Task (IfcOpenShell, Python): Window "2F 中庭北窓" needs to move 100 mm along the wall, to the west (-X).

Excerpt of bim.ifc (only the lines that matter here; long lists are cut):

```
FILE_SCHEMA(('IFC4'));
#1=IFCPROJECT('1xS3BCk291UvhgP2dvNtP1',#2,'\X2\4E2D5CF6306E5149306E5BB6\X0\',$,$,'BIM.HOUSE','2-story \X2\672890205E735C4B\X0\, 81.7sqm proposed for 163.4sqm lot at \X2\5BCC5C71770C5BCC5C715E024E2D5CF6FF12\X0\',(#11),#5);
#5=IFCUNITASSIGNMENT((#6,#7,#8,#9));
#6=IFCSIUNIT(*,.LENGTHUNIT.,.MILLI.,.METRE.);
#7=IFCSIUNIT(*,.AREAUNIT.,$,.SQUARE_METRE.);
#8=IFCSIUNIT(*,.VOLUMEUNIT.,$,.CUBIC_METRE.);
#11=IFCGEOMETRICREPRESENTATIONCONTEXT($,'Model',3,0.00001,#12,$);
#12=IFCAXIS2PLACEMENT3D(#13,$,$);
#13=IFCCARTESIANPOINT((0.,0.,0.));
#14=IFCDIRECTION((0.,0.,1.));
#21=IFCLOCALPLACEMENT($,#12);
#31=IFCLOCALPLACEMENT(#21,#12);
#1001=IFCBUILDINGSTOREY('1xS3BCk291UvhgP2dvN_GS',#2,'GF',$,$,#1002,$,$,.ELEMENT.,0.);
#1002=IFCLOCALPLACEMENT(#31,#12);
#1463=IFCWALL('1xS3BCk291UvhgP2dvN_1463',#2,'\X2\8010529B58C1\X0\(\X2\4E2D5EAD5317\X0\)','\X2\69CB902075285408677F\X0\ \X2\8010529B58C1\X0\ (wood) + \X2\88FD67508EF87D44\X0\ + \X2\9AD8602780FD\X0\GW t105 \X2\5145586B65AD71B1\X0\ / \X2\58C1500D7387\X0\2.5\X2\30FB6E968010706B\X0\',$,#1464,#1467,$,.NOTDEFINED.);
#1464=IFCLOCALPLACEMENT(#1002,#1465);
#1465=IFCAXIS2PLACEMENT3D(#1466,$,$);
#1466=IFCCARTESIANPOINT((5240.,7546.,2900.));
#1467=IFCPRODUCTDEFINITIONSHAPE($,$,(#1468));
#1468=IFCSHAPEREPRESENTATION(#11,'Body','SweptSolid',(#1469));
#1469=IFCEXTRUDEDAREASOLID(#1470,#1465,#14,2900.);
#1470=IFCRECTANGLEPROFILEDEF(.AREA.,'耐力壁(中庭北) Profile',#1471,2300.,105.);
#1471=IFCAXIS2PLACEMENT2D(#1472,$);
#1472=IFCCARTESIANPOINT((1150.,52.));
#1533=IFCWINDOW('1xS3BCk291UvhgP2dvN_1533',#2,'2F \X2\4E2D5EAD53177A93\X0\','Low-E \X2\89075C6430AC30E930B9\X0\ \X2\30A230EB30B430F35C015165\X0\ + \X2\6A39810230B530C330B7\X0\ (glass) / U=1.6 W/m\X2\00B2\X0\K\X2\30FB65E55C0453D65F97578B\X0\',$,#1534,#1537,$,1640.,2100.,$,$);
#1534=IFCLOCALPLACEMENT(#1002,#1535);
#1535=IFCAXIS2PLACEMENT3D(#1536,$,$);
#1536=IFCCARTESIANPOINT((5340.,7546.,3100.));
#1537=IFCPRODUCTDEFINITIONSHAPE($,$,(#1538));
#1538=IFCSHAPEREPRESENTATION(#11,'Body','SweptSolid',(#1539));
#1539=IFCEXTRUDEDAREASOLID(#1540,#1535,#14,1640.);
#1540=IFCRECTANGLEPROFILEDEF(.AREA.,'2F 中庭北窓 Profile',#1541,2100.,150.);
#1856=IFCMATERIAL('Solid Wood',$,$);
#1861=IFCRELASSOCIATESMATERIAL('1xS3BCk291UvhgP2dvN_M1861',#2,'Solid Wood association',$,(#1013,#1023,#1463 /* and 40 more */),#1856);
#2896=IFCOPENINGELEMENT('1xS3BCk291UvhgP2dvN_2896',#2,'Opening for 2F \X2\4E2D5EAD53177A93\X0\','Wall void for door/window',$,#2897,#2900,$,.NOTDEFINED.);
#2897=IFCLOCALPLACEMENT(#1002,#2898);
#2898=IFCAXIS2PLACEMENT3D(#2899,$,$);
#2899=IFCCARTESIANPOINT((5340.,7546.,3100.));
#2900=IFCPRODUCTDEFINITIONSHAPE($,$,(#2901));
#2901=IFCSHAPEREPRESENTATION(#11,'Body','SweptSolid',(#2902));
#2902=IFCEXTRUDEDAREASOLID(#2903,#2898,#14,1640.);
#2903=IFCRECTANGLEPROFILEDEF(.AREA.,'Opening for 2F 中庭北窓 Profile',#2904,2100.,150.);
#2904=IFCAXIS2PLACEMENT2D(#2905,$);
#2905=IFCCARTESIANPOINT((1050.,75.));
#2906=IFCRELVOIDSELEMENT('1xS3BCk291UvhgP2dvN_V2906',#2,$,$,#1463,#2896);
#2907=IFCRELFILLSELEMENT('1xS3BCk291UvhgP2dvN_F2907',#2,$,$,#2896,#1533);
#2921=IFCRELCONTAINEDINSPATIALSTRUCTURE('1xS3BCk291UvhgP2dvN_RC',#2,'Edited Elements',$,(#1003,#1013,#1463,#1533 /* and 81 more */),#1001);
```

```python
import ifcopenshell
import ifcopenshell.api.geometry
import ifcopenshell.util.placement
import ifcopenshell.util.unit

model = ifcopenshell.open("bim.ifc")
unit_scale = ifcopenshell.util.unit.calculate_unit_scale(model)

window = model.by_id(1533)
opening = window.FillsVoids[0].RelatingOpeningElement
wall = opening.VoidsElements[0].RelatingBuildingElement

wall_matrix = ifcopenshell.util.placement.get_local_placement(wall.ObjectPlacement)
shift = wall_matrix[:3, 0] * -0.1 / unit_scale
before = ifcopenshell.util.placement.get_local_placement(window.ObjectPlacement)[:3, 3].copy()

# The window is not placed relative to its opening, so move both.
for product in (opening, window):
    matrix = ifcopenshell.util.placement.get_local_placement(product.ObjectPlacement)
    matrix[:3, 3] += shift
    ifcopenshell.api.geometry.edit_object_placement(model, product=product, matrix=matrix, is_si=False)

after = ifcopenshell.util.placement.get_local_placement(window.ObjectPlacement)[:3, 3]
print("window moved by", (after - before).round(3) + 0.0)

model.write("bim_edited.ifc")
```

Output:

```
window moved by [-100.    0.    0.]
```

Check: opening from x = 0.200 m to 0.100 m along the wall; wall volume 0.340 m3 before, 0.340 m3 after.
